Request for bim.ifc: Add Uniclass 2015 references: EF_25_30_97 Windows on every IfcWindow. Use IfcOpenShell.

First a look at what the model holds.

```python
import ifcopenshell

model = ifcopenshell.open("bim.ifc")
print(model.schema)
print("classifications:", [c.Name for c in model.by_type("IfcClassification")])
for ifc_class in ("IfcDoor", "IfcRoof", "IfcStair", "IfcWall", "IfcWindow"):
    print(ifc_class, len(model.by_type(ifc_class)))
```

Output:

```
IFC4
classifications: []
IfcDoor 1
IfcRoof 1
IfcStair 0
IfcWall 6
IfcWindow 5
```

```python
import ifcopenshell
import ifcopenshell.api.classification

model = ifcopenshell.open("bim.ifc")

system = ifcopenshell.api.classification.add_classification(model, classification="Uniclass 2015")

codes = {
    "IfcWindow": ("EF_25_30_97", "Windows"),
}
for ifc_class, (code, name) in codes.items():
    products = model.by_type(ifc_class)
    ifcopenshell.api.classification.add_reference(
        model, products=products, classification=system, identification=code, name=name
    )
    print(code, len(products))

model.write("bim_edited.ifc")
```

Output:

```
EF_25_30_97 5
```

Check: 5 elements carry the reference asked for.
